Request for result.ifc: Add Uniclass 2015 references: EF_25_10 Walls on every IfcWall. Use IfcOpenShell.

First a look at what the model holds.

```python
import ifcopenshell

model = ifcopenshell.open("result.ifc")
print(model.schema)
print("classifications:", [c.Name for c in model.by_type("IfcClassification")])
for ifc_class in ("IfcDoor", "IfcRoof", "IfcStair", "IfcWall", "IfcWindow"):
    print(ifc_class, len(model.by_type(ifc_class)))
```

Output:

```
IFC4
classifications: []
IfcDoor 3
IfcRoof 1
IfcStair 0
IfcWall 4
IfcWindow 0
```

```python
import ifcopenshell
import ifcopenshell.api.classification

model = ifcopenshell.open("result.ifc")

system = ifcopenshell.api.classification.add_classification(model, classification="Uniclass 2015")

codes = {
    "IfcWall": ("EF_25_10", "Walls"),
}
for ifc_class, (code, name) in codes.items():
    products = model.by_type(ifc_class)
    ifcopenshell.api.classification.add_reference(
        model, products=products, classification=system, identification=code, name=name
    )
    print(code, len(products))

model.write("result_v2.ifc")
```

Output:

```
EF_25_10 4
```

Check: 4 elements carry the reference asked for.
